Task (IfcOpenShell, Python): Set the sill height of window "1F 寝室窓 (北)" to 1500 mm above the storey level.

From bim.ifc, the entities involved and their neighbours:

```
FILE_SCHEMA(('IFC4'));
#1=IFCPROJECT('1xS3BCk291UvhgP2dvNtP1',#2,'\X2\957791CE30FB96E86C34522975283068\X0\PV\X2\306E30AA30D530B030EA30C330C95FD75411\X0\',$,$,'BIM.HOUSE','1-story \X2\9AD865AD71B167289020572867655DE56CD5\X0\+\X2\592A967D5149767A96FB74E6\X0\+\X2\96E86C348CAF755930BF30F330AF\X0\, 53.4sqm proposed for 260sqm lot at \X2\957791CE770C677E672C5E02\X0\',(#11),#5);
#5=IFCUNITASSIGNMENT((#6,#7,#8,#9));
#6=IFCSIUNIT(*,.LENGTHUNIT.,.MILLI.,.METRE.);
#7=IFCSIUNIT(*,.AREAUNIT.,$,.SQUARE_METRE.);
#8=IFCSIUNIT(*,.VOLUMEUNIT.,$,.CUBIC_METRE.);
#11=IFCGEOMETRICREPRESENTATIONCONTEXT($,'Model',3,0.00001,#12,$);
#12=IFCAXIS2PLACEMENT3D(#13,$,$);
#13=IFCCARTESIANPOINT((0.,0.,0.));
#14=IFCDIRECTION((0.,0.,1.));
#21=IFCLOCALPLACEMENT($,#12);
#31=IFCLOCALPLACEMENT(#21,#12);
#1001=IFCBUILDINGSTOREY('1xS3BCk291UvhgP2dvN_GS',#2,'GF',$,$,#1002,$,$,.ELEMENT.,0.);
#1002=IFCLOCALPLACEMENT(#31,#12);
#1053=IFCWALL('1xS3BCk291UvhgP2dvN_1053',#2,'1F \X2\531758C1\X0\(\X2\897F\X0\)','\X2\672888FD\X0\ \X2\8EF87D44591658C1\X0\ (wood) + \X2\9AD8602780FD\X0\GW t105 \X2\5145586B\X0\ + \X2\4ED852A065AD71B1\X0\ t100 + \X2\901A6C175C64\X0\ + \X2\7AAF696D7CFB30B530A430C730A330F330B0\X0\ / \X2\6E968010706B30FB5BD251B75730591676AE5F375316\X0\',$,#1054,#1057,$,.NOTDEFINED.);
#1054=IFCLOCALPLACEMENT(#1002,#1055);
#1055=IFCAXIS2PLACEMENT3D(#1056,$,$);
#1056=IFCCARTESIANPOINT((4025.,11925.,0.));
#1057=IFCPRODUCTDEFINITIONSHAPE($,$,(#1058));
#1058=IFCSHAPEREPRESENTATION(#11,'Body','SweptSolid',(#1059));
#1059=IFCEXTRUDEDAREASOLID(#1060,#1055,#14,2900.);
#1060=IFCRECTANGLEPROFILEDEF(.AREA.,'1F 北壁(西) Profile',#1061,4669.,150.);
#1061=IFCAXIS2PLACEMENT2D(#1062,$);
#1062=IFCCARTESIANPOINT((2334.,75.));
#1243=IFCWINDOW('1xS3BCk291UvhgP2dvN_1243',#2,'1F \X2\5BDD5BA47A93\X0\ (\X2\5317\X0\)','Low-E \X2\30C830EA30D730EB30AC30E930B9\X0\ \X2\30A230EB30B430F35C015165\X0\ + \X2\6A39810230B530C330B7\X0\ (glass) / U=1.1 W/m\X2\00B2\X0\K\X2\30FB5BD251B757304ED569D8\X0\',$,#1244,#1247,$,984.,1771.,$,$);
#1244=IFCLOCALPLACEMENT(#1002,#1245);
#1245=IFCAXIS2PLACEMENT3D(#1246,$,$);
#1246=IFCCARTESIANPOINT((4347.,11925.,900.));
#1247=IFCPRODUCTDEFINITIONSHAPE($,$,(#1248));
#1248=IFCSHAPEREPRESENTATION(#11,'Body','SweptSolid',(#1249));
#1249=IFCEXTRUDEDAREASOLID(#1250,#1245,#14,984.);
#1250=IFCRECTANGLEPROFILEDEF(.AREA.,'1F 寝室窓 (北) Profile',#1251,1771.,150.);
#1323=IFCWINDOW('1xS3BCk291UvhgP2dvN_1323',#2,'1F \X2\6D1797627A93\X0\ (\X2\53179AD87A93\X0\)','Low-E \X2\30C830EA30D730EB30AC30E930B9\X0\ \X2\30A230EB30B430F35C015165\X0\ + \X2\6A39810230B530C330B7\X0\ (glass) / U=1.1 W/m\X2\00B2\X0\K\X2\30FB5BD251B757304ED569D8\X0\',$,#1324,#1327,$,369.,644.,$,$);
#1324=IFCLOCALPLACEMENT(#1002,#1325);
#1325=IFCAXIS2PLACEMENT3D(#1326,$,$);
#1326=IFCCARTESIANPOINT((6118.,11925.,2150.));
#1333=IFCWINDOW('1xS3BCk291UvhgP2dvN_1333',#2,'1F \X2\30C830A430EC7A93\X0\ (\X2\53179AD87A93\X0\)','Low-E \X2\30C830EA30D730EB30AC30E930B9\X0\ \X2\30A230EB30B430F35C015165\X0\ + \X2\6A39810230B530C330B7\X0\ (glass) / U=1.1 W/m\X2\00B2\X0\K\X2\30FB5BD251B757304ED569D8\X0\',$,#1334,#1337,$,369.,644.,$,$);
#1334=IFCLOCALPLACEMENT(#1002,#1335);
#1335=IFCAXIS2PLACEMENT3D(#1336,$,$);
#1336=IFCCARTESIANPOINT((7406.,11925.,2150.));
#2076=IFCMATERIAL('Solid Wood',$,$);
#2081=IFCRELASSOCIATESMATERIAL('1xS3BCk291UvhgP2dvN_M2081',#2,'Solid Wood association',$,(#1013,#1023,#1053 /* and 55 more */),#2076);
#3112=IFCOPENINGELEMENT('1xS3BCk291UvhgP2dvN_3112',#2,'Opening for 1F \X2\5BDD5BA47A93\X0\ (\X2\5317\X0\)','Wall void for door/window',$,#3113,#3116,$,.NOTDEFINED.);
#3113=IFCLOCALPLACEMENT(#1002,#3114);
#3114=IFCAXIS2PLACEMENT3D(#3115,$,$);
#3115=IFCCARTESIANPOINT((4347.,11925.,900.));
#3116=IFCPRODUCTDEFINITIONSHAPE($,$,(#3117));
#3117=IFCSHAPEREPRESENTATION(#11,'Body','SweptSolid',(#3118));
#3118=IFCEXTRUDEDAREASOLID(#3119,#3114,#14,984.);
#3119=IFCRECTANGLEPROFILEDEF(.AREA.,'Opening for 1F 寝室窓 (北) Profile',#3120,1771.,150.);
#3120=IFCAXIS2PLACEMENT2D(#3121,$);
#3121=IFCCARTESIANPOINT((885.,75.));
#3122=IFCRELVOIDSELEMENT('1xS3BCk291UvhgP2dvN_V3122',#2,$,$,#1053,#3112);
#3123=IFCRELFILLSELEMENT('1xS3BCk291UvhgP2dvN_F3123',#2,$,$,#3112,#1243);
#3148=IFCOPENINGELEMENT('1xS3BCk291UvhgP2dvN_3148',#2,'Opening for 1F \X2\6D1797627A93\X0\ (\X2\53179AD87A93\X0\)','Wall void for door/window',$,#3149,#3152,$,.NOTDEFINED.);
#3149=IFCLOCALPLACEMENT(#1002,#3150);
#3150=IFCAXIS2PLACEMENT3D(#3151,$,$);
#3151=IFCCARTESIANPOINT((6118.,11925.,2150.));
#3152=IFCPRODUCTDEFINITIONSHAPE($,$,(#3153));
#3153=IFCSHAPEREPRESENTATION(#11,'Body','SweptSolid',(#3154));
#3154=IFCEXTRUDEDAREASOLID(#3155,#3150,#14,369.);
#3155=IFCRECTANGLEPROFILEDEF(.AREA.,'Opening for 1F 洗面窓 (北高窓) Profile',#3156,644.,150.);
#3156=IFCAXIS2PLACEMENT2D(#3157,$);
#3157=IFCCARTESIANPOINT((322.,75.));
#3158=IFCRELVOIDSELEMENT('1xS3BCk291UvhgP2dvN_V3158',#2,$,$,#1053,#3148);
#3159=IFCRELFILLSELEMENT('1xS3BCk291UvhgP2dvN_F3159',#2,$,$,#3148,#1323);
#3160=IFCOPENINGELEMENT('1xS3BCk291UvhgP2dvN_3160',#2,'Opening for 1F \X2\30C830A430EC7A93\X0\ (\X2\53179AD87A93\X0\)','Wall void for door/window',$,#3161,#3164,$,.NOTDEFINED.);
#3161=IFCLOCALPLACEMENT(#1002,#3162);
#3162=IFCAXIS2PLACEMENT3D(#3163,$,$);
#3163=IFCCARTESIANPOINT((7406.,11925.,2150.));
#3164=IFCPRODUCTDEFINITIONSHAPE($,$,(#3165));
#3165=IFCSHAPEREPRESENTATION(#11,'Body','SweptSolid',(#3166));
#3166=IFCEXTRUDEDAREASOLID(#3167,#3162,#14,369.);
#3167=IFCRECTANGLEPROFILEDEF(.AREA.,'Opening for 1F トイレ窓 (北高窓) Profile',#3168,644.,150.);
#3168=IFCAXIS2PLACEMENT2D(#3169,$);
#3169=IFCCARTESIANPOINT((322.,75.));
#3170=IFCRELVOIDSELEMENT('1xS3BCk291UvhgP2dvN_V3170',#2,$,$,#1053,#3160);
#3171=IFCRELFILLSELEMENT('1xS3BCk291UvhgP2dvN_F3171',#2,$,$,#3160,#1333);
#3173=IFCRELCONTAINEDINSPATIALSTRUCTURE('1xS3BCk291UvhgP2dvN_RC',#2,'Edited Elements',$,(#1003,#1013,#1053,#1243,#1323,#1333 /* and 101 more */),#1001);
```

```python
import numpy as np
import ifcopenshell
import ifcopenshell.api.geometry
import ifcopenshell.geom
import ifcopenshell.util.element
import ifcopenshell.util.placement
import ifcopenshell.util.shape
import ifcopenshell.util.unit

model = ifcopenshell.open("bim.ifc")
unit_scale = ifcopenshell.util.unit.calculate_unit_scale(model)

window = model.by_guid("1xS3BCk291UvhgP2dvN_1243")
opening = window.FillsVoids[0].RelatingOpeningElement
storey = ifcopenshell.util.element.get_container(window, ifc_class="IfcBuildingStorey")
level = ifcopenshell.util.placement.get_local_placement(storey.ObjectPlacement)[2, 3]

# The opening's origin need not be at the sill, so measure its lowest point.
shape = ifcopenshell.geom.create_shape(ifcopenshell.geom.settings(), opening)
bottom = ifcopenshell.util.shape.get_shape_bottom_elevation(shape, shape.geometry) / unit_scale
dz = level + 1500.0 - bottom

shift = np.array([0.0, 0.0, dz])
# The window is not placed relative to its opening, so move both.
for product in (opening, window):
    matrix = ifcopenshell.util.placement.get_local_placement(product.ObjectPlacement)
    matrix[:3, 3] += shift
    ifcopenshell.api.geometry.edit_object_placement(model, product=product, matrix=matrix, is_si=False)

print(f"moved by {dz * unit_scale:+.3f} m")

model.write("bim_edited.ifc")
```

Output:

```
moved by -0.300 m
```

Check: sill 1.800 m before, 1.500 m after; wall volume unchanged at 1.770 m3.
